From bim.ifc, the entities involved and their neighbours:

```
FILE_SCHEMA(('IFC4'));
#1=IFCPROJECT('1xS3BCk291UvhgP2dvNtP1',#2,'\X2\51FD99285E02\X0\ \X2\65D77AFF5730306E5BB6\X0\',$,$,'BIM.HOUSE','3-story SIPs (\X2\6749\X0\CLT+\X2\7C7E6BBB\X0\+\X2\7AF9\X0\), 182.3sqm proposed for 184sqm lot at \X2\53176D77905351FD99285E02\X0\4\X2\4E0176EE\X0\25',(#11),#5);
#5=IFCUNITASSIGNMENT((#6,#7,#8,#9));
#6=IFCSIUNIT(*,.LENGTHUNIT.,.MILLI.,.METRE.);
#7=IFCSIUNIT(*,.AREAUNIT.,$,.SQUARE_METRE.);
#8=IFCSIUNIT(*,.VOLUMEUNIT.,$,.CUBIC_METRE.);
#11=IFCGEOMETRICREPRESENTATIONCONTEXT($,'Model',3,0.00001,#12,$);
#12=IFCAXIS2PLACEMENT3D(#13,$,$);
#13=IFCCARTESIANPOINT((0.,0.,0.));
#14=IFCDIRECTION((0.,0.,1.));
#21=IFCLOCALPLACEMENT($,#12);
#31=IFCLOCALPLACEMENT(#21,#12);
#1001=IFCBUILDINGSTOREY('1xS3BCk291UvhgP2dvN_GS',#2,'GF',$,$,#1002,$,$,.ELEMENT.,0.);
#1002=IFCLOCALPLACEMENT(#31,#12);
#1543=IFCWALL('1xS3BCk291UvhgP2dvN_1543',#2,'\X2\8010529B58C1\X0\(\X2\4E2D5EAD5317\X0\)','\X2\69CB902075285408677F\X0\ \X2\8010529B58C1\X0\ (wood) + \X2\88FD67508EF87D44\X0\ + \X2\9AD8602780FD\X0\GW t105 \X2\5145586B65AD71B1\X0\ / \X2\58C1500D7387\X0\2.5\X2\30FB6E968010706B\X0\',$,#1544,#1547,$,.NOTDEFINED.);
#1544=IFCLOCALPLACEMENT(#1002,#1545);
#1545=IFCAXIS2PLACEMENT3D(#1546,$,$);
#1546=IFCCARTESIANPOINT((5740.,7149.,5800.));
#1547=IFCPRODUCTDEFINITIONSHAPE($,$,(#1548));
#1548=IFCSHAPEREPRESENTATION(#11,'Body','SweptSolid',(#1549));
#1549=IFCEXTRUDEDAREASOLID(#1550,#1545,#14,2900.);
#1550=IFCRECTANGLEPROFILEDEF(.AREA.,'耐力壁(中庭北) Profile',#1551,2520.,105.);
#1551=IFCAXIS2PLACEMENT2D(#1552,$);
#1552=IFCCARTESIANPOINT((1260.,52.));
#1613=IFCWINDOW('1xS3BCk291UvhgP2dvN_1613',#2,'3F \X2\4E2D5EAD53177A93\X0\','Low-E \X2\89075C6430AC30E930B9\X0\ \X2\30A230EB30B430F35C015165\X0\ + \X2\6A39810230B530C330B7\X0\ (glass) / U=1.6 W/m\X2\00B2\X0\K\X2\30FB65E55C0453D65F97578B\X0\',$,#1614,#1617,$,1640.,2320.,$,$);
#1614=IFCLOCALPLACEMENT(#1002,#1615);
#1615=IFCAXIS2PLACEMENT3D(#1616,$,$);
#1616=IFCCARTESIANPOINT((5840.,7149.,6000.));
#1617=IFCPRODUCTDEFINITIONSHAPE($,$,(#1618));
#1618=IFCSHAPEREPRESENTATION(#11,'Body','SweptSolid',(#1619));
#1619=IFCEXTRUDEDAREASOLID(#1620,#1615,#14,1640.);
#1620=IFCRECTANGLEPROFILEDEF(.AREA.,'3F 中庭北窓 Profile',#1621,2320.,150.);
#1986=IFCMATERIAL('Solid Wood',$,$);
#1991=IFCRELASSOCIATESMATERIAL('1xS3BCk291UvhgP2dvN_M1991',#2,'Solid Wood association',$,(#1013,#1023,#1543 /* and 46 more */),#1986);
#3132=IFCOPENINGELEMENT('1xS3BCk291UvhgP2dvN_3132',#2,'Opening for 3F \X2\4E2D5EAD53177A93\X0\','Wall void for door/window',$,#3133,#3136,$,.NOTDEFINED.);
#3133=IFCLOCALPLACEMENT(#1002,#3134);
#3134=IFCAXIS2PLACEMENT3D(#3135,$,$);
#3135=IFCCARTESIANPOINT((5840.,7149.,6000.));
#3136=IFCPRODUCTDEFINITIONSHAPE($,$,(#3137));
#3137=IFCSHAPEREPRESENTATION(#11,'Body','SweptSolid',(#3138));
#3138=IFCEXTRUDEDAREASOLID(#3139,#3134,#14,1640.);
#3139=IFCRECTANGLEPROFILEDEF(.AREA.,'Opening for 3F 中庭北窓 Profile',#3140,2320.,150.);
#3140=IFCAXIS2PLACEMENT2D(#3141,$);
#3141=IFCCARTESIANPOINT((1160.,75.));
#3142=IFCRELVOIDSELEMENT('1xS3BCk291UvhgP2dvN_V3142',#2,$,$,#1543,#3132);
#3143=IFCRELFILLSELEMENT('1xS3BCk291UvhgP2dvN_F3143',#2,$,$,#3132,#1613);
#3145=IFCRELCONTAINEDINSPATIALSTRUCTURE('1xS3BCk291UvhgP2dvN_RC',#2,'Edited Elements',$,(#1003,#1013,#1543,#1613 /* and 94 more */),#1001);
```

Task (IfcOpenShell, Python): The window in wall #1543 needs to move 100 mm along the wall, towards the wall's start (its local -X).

```python
import ifcopenshell
import ifcopenshell.api.geometry
import ifcopenshell.util.placement
import ifcopenshell.util.unit

model = ifcopenshell.open("bim.ifc")
unit_scale = ifcopenshell.util.unit.calculate_unit_scale(model)

window = model.by_guid("1xS3BCk291UvhgP2dvN_1613")
opening = window.FillsVoids[0].RelatingOpeningElement
wall = opening.VoidsElements[0].RelatingBuildingElement

wall_matrix = ifcopenshell.util.placement.get_local_placement(wall.ObjectPlacement)
shift = wall_matrix[:3, 0] * -0.1 / unit_scale
before = ifcopenshell.util.placement.get_local_placement(window.ObjectPlacement)[:3, 3].copy()

# The window is not placed relative to its opening, so move both.
for product in (opening, window):
    matrix = ifcopenshell.util.placement.get_local_placement(product.ObjectPlacement)
    matrix[:3, 3] += shift
    ifcopenshell.api.geometry.edit_object_placement(model, product=product, matrix=matrix, is_si=False)

after = ifcopenshell.util.placement.get_local_placement(window.ObjectPlacement)[:3, 3]
print("window moved by", (after - before).round(3) + 0.0)

model.write("bim_v2.ifc")
```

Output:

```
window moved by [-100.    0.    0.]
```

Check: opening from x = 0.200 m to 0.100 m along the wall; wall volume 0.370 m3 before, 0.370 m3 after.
